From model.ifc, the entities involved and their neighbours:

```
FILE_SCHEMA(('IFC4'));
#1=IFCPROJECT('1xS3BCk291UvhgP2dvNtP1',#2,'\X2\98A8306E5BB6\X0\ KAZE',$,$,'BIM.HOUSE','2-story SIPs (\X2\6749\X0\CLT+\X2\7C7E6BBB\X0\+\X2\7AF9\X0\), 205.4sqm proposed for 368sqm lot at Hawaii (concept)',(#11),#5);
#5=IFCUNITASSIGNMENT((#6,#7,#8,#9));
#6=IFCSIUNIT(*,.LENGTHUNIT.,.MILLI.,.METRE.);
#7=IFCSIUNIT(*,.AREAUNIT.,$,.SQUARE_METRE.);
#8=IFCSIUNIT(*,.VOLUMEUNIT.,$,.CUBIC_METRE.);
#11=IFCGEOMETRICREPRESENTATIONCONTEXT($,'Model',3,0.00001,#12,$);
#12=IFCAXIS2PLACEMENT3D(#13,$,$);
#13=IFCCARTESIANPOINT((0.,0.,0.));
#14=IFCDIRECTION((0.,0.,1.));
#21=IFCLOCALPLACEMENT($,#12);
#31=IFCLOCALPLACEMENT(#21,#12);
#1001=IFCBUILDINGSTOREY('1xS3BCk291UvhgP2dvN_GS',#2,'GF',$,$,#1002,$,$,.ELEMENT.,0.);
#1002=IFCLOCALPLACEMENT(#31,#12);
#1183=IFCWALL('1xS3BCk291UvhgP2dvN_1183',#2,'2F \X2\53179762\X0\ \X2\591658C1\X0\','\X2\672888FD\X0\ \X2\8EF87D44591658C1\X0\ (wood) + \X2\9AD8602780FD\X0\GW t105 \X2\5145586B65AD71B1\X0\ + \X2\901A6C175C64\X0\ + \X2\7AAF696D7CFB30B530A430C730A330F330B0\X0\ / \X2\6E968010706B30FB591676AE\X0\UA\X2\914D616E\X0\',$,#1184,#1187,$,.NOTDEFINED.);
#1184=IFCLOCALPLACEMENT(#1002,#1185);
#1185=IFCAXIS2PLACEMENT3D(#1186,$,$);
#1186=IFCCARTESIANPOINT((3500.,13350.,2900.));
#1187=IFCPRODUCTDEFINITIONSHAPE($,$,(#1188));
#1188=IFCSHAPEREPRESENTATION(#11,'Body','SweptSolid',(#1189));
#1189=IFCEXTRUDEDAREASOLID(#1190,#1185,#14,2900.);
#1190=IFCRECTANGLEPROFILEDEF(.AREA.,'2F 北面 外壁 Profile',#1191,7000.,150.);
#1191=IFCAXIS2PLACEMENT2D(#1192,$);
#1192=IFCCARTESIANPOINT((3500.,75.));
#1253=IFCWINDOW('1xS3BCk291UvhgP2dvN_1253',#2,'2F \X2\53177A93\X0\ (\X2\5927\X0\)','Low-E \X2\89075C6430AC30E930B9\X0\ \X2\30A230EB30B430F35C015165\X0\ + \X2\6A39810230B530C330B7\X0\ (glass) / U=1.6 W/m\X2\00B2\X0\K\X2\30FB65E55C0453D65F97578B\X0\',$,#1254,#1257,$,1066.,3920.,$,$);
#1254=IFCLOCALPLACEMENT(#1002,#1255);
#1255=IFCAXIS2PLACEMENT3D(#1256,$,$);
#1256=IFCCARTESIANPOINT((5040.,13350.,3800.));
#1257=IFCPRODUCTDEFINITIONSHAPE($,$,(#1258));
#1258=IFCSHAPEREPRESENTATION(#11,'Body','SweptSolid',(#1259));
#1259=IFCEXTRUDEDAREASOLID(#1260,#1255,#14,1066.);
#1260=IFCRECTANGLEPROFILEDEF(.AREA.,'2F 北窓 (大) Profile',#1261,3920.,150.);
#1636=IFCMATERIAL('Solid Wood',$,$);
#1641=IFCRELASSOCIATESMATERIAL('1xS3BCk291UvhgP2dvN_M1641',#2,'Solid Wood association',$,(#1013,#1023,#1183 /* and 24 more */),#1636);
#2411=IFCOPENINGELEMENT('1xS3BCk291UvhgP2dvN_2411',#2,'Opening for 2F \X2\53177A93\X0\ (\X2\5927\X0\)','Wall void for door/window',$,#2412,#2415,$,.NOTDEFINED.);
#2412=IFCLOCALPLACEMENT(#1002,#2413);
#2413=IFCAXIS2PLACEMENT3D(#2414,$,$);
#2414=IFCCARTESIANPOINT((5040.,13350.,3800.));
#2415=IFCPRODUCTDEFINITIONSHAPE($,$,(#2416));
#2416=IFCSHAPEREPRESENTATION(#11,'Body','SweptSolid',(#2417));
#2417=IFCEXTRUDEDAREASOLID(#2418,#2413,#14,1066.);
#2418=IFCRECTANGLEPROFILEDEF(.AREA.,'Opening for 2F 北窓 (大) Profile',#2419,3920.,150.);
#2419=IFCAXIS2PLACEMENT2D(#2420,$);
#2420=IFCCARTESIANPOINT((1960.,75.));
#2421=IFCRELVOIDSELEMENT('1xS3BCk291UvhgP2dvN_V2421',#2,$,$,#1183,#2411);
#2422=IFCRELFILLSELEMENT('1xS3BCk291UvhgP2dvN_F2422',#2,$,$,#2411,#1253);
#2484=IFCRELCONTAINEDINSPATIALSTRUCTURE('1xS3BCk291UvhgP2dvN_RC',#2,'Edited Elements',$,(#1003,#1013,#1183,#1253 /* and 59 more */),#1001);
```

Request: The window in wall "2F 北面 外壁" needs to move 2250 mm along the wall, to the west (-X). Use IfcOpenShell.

```python
import ifcopenshell
import ifcopenshell.api.geometry
import ifcopenshell.util.placement

model = ifcopenshell.open("model.ifc")

window = model.by_guid("1xS3BCk291UvhgP2dvN_1253")
opening = window.FillsVoids[0].RelatingOpeningElement
wall = opening.VoidsElements[0].RelatingBuildingElement

wall_matrix = ifcopenshell.util.placement.get_local_placement(wall.ObjectPlacement)
shift = wall_matrix[:3, 0] * -2250.0
before = ifcopenshell.util.placement.get_local_placement(window.ObjectPlacement)[:3, 3].copy()

# The window is not placed relative to its opening, so move both.
for product in (opening, window):
    matrix = ifcopenshell.util.placement.get_local_placement(product.ObjectPlacement)
    matrix[:3, 3] += shift
    ifcopenshell.api.geometry.edit_object_placement(model, product=product, matrix=matrix, is_si=False)

after = ifcopenshell.util.placement.get_local_placement(window.ObjectPlacement)[:3, 3]
print("window moved by", (after - before).round(3) + 0.0)

model.write("model_edited.ifc")
```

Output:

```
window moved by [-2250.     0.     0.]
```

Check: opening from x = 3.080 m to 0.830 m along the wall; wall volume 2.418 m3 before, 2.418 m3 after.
